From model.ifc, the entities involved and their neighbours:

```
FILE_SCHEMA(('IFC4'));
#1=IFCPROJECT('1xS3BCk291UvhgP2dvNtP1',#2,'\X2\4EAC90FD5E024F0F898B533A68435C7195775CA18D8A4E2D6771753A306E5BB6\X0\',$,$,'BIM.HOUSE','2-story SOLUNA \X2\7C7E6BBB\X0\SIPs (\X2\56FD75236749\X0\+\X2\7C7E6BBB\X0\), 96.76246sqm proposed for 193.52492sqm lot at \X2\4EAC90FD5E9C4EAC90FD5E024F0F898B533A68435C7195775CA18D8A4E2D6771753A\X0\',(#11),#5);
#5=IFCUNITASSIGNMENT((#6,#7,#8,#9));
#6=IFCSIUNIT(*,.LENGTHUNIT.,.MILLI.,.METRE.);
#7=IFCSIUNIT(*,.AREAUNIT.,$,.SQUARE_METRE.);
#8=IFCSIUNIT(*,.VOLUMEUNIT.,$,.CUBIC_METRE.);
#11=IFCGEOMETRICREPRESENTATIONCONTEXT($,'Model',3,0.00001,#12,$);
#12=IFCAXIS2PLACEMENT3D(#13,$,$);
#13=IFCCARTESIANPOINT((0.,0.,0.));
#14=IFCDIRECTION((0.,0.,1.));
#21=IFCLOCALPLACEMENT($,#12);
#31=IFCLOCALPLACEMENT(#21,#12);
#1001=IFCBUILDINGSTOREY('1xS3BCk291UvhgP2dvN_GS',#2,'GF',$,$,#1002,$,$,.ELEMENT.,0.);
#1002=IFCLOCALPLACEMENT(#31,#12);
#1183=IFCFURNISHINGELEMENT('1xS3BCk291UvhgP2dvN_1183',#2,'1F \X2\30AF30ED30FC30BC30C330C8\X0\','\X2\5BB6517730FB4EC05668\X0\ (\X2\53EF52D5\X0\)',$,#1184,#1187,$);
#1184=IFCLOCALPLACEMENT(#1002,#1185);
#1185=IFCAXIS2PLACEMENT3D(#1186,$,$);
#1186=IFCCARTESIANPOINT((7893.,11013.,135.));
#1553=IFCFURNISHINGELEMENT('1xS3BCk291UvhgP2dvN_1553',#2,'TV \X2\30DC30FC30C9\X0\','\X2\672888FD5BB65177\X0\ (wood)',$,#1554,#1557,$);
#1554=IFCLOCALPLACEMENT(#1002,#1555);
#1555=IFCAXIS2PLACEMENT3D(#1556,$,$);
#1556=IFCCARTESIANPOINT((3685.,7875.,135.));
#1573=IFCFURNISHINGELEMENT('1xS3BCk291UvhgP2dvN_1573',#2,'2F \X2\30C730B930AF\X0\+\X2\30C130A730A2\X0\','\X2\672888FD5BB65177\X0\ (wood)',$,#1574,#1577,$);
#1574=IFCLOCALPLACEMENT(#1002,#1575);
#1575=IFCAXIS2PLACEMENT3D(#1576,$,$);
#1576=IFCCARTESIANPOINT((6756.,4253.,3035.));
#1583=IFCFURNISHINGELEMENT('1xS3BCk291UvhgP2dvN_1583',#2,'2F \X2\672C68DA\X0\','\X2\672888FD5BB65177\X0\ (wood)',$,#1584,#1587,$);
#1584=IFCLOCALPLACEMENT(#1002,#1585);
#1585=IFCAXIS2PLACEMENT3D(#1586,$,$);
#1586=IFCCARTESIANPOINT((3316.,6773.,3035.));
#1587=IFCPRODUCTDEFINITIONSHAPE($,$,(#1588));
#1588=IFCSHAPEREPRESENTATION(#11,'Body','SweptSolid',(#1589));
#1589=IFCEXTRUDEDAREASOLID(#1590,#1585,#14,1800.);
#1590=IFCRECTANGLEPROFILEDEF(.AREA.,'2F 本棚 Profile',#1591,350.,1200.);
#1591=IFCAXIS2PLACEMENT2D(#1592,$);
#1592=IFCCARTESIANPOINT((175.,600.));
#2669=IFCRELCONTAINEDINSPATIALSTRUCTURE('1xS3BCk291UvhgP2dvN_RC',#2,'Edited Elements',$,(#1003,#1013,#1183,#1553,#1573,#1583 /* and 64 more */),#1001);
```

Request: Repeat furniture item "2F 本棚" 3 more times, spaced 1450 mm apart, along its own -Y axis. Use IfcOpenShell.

```python
import ifcopenshell
import ifcopenshell.api.geometry
import ifcopenshell.api.root
import ifcopenshell.util.element
import ifcopenshell.util.placement
import ifcopenshell.util.unit

model = ifcopenshell.open("model.ifc")
unit_scale = ifcopenshell.util.unit.calculate_unit_scale(model)


def reuse_history(source, copy):
    """copy_class also copies each property set's owner history, people and application; keep the originals."""
    for rel in copy.IsDefinedBy:
        if rel.is_a("IfcRelDefinesByProperties") and (history := rel.RelatingPropertyDefinition.OwnerHistory):
            rel.RelatingPropertyDefinition.OwnerHistory = source.OwnerHistory
            ifcopenshell.util.element.remove_deep2(model, history)


source = model.by_guid("1xS3BCk291UvhgP2dvN_1583")
base = ifcopenshell.util.placement.get_local_placement(source.ObjectPlacement)
step = -base[:3, 1] * 1.45 / unit_scale

for i in range(1, 4):
    copy = ifcopenshell.api.root.copy_class(model, product=source)
    copy.Representation = ifcopenshell.util.element.copy_deep(
        model, source.Representation, exclude=["IfcGeometricRepresentationContext", "IfcRepresentationMap"]
    )
    reuse_history(source, copy)
    matrix = base.copy()
    matrix[:3, 3] += i * step
    print("added at", matrix[:3, 3].round(3) + 0.0)
    ifcopenshell.api.geometry.edit_object_placement(model, product=copy, matrix=matrix, is_si=False)

model.write("model_rev.ifc")
```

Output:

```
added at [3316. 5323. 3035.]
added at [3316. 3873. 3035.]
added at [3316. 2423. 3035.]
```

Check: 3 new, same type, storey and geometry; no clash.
